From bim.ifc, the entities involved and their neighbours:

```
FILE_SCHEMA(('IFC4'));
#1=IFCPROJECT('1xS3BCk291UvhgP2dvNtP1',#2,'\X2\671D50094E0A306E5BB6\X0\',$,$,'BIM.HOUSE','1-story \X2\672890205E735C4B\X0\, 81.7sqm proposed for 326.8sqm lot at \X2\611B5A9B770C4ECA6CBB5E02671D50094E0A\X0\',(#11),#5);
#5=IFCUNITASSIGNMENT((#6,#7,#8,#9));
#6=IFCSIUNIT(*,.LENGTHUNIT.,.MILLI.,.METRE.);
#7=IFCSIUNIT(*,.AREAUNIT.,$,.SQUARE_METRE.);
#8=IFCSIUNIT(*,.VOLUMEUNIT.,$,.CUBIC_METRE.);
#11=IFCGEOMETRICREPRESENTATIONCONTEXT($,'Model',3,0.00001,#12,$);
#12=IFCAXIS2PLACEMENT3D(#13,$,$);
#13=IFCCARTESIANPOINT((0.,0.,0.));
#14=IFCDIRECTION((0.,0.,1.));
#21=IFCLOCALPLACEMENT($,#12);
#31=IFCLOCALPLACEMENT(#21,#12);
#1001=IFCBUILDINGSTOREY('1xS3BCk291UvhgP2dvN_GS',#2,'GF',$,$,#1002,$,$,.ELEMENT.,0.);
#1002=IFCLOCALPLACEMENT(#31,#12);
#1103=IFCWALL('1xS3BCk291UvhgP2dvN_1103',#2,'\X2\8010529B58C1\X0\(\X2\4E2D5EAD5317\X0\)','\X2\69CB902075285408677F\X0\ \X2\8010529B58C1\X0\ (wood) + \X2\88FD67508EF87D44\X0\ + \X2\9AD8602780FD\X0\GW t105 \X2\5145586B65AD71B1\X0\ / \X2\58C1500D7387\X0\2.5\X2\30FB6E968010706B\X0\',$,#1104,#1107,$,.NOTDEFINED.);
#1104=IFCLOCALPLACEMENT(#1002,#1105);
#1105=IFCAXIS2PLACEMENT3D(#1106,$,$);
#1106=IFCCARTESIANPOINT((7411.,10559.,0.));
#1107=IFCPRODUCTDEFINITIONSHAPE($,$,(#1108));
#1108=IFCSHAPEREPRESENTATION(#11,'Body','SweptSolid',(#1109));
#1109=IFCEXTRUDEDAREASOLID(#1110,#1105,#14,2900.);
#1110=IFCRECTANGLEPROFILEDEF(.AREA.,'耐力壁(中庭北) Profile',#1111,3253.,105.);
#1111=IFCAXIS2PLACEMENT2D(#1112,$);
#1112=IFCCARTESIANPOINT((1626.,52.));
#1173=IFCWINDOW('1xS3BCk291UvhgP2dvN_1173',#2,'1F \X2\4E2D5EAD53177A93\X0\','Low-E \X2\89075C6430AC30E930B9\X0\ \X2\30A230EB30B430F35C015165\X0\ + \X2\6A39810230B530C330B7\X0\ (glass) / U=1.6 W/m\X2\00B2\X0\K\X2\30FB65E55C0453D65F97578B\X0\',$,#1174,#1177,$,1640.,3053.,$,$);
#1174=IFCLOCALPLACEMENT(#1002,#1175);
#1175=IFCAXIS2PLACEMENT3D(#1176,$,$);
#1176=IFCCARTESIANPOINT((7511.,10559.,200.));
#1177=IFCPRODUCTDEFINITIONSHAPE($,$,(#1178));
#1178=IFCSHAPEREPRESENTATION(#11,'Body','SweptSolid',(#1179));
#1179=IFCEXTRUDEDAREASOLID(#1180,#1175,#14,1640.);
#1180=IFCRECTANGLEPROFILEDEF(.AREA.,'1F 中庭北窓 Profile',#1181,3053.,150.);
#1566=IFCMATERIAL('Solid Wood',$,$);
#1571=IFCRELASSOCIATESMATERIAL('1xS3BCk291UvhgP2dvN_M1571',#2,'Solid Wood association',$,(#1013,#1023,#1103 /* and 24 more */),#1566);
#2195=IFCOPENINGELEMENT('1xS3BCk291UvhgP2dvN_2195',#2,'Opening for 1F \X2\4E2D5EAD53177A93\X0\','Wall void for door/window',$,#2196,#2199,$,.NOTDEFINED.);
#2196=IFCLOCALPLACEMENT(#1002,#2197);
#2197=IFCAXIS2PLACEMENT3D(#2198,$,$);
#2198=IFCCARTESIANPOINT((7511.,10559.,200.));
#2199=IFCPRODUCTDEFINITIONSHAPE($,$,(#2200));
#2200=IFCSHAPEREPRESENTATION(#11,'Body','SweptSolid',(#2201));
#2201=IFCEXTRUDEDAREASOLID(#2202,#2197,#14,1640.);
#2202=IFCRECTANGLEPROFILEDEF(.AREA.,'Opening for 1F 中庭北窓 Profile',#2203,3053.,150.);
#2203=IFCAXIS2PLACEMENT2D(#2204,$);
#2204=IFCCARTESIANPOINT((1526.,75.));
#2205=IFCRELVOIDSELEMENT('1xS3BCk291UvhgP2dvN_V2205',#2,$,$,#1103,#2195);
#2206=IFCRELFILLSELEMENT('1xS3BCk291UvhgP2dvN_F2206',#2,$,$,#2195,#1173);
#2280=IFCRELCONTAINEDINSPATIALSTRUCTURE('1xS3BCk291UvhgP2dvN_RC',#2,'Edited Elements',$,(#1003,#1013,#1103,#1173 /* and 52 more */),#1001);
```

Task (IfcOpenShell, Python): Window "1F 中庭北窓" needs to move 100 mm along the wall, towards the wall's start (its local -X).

```python
import ifcopenshell
import ifcopenshell.api.geometry
import ifcopenshell.util.placement
import ifcopenshell.util.unit

model = ifcopenshell.open("bim.ifc")
unit_scale = ifcopenshell.util.unit.calculate_unit_scale(model)

window = model.by_guid("1xS3BCk291UvhgP2dvN_1173")
opening = window.FillsVoids[0].RelatingOpeningElement
wall = opening.VoidsElements[0].RelatingBuildingElement

wall_matrix = ifcopenshell.util.placement.get_local_placement(wall.ObjectPlacement)
shift = wall_matrix[:3, 0] * -0.1 / unit_scale
before = ifcopenshell.util.placement.get_local_placement(window.ObjectPlacement)[:3, 3].copy()

# The window is not placed relative to its opening, so move both.
for product in (opening, window):
    matrix = ifcopenshell.util.placement.get_local_placement(product.ObjectPlacement)
    matrix[:3, 3] += shift
    ifcopenshell.api.geometry.edit_object_placement(model, product=product, matrix=matrix, is_si=False)

after = ifcopenshell.util.placement.get_local_placement(window.ObjectPlacement)[:3, 3]
print("window moved by", (after - before).round(3) + 0.0)

model.write("bim_v2.ifc")
```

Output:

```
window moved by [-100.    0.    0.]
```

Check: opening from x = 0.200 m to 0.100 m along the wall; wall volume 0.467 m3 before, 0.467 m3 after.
